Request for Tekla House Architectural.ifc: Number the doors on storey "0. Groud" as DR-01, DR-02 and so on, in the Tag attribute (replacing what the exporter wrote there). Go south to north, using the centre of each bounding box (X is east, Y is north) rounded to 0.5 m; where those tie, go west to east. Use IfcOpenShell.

First a look at what the model holds.

```python
import ifcopenshell
import ifcopenshell.util.element
import ifcopenshell.util.placement

model = ifcopenshell.open("Tekla House Architectural.ifc")
print(model.schema)
storey = next(s for s in model.by_type("IfcBuildingStorey") if s.Name == "0. Groud")
doors = [e for e in ifcopenshell.util.element.get_decomposition(storey) if e.is_a("IfcDoor")]
for e in sorted(doors, key=lambda e: e.id()):
    origin = ifcopenshell.util.placement.get_local_placement(e.ObjectPlacement)[:3, 3]
    print(e.id(), e.Tag, e.Name, origin.round(2) + 0.0, sep=" | ")
```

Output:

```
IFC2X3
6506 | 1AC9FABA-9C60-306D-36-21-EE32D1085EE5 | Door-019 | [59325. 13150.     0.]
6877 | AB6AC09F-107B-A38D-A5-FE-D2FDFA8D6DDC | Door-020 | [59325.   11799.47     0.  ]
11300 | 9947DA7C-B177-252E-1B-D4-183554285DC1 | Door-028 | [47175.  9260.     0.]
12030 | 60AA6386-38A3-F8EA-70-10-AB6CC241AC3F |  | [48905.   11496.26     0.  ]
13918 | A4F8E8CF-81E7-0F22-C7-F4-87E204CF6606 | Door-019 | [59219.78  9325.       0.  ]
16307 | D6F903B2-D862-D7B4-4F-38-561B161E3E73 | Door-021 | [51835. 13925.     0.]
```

```python
import ifcopenshell
import ifcopenshell.geom
import ifcopenshell.util.element
import ifcopenshell.util.shape

model = ifcopenshell.open("Tekla House Architectural.ifc")
settings = ifcopenshell.geom.settings()
settings.set("use-world-coords", True)


def centre(element):
    shape = ifcopenshell.geom.create_shape(settings, element)
    return ifcopenshell.util.shape.get_bbox_centroid(shape.geometry)


storey = next(s for s in model.by_type("IfcBuildingStorey") if s.Name == "0. Groud")
doors = [e for e in ifcopenshell.util.element.get_decomposition(storey) if e.is_a("IfcDoor")]

# Insertion points can sit at a corner or the storey origin, so sort by the geometry (in metres).
centres = {e: centre(e) for e in doors}
doors.sort(key=lambda e: (round(centres[e][1] / 0.5), centres[e][0]))

for i, e in enumerate(doors, start=1):
    number = f"DR-{i:02d}"
    e.Tag = number
    print(e.id(), number)

model.write("Tekla House Architectural_updated.ifc")
```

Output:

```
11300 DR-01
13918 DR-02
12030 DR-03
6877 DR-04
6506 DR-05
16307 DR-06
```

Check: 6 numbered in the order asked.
